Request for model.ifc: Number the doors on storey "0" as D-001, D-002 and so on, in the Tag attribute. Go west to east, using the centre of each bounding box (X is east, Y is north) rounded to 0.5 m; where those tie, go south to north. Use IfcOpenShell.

First a look at what the model holds.

```python
import ifcopenshell
import ifcopenshell.util.element
import ifcopenshell.util.placement

model = ifcopenshell.open("model.ifc")
print(model.schema)
storey = next(s for s in model.by_type("IfcBuildingStorey") if s.Name == "0")
doors = [e for e in ifcopenshell.util.element.get_decomposition(storey) if e.is_a("IfcDoor")]
for e in sorted(doors, key=lambda e: e.id()):
    origin = ifcopenshell.util.placement.get_local_placement(e.ObjectPlacement)[:3, 3]
    print(e.id(), e.Tag, e.Name, origin.round(2) + 0.0, sep=" | ")
```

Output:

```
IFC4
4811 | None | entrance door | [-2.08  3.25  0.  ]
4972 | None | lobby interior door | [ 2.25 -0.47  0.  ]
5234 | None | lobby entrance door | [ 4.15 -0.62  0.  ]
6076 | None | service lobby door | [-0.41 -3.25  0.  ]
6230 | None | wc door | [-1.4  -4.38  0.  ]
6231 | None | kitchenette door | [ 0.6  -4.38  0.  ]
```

```python
import ifcopenshell
import ifcopenshell.geom
import ifcopenshell.util.element
import ifcopenshell.util.shape

model = ifcopenshell.open("model.ifc")
settings = ifcopenshell.geom.settings()
settings.set("use-world-coords", True)


def centre(element):
    shape = ifcopenshell.geom.create_shape(settings, element)
    return ifcopenshell.util.shape.get_bbox_centroid(shape.geometry)


storey = next(s for s in model.by_type("IfcBuildingStorey") if s.Name == "0")
doors = [e for e in ifcopenshell.util.element.get_decomposition(storey) if e.is_a("IfcDoor")]

# Insertion points can sit at a corner or the storey origin, so sort by the geometry (in metres).
centres = {e: centre(e) for e in doors}
doors.sort(key=lambda e: (round(centres[e][0] / 0.5), centres[e][1]))

for i, e in enumerate(doors, start=1):
    number = f"D-0{i:02d}"
    e.Tag = number
    print(e.id(), number)

model.write("model_v2.ifc")
```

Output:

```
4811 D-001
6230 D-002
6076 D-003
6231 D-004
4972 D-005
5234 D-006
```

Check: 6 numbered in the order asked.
